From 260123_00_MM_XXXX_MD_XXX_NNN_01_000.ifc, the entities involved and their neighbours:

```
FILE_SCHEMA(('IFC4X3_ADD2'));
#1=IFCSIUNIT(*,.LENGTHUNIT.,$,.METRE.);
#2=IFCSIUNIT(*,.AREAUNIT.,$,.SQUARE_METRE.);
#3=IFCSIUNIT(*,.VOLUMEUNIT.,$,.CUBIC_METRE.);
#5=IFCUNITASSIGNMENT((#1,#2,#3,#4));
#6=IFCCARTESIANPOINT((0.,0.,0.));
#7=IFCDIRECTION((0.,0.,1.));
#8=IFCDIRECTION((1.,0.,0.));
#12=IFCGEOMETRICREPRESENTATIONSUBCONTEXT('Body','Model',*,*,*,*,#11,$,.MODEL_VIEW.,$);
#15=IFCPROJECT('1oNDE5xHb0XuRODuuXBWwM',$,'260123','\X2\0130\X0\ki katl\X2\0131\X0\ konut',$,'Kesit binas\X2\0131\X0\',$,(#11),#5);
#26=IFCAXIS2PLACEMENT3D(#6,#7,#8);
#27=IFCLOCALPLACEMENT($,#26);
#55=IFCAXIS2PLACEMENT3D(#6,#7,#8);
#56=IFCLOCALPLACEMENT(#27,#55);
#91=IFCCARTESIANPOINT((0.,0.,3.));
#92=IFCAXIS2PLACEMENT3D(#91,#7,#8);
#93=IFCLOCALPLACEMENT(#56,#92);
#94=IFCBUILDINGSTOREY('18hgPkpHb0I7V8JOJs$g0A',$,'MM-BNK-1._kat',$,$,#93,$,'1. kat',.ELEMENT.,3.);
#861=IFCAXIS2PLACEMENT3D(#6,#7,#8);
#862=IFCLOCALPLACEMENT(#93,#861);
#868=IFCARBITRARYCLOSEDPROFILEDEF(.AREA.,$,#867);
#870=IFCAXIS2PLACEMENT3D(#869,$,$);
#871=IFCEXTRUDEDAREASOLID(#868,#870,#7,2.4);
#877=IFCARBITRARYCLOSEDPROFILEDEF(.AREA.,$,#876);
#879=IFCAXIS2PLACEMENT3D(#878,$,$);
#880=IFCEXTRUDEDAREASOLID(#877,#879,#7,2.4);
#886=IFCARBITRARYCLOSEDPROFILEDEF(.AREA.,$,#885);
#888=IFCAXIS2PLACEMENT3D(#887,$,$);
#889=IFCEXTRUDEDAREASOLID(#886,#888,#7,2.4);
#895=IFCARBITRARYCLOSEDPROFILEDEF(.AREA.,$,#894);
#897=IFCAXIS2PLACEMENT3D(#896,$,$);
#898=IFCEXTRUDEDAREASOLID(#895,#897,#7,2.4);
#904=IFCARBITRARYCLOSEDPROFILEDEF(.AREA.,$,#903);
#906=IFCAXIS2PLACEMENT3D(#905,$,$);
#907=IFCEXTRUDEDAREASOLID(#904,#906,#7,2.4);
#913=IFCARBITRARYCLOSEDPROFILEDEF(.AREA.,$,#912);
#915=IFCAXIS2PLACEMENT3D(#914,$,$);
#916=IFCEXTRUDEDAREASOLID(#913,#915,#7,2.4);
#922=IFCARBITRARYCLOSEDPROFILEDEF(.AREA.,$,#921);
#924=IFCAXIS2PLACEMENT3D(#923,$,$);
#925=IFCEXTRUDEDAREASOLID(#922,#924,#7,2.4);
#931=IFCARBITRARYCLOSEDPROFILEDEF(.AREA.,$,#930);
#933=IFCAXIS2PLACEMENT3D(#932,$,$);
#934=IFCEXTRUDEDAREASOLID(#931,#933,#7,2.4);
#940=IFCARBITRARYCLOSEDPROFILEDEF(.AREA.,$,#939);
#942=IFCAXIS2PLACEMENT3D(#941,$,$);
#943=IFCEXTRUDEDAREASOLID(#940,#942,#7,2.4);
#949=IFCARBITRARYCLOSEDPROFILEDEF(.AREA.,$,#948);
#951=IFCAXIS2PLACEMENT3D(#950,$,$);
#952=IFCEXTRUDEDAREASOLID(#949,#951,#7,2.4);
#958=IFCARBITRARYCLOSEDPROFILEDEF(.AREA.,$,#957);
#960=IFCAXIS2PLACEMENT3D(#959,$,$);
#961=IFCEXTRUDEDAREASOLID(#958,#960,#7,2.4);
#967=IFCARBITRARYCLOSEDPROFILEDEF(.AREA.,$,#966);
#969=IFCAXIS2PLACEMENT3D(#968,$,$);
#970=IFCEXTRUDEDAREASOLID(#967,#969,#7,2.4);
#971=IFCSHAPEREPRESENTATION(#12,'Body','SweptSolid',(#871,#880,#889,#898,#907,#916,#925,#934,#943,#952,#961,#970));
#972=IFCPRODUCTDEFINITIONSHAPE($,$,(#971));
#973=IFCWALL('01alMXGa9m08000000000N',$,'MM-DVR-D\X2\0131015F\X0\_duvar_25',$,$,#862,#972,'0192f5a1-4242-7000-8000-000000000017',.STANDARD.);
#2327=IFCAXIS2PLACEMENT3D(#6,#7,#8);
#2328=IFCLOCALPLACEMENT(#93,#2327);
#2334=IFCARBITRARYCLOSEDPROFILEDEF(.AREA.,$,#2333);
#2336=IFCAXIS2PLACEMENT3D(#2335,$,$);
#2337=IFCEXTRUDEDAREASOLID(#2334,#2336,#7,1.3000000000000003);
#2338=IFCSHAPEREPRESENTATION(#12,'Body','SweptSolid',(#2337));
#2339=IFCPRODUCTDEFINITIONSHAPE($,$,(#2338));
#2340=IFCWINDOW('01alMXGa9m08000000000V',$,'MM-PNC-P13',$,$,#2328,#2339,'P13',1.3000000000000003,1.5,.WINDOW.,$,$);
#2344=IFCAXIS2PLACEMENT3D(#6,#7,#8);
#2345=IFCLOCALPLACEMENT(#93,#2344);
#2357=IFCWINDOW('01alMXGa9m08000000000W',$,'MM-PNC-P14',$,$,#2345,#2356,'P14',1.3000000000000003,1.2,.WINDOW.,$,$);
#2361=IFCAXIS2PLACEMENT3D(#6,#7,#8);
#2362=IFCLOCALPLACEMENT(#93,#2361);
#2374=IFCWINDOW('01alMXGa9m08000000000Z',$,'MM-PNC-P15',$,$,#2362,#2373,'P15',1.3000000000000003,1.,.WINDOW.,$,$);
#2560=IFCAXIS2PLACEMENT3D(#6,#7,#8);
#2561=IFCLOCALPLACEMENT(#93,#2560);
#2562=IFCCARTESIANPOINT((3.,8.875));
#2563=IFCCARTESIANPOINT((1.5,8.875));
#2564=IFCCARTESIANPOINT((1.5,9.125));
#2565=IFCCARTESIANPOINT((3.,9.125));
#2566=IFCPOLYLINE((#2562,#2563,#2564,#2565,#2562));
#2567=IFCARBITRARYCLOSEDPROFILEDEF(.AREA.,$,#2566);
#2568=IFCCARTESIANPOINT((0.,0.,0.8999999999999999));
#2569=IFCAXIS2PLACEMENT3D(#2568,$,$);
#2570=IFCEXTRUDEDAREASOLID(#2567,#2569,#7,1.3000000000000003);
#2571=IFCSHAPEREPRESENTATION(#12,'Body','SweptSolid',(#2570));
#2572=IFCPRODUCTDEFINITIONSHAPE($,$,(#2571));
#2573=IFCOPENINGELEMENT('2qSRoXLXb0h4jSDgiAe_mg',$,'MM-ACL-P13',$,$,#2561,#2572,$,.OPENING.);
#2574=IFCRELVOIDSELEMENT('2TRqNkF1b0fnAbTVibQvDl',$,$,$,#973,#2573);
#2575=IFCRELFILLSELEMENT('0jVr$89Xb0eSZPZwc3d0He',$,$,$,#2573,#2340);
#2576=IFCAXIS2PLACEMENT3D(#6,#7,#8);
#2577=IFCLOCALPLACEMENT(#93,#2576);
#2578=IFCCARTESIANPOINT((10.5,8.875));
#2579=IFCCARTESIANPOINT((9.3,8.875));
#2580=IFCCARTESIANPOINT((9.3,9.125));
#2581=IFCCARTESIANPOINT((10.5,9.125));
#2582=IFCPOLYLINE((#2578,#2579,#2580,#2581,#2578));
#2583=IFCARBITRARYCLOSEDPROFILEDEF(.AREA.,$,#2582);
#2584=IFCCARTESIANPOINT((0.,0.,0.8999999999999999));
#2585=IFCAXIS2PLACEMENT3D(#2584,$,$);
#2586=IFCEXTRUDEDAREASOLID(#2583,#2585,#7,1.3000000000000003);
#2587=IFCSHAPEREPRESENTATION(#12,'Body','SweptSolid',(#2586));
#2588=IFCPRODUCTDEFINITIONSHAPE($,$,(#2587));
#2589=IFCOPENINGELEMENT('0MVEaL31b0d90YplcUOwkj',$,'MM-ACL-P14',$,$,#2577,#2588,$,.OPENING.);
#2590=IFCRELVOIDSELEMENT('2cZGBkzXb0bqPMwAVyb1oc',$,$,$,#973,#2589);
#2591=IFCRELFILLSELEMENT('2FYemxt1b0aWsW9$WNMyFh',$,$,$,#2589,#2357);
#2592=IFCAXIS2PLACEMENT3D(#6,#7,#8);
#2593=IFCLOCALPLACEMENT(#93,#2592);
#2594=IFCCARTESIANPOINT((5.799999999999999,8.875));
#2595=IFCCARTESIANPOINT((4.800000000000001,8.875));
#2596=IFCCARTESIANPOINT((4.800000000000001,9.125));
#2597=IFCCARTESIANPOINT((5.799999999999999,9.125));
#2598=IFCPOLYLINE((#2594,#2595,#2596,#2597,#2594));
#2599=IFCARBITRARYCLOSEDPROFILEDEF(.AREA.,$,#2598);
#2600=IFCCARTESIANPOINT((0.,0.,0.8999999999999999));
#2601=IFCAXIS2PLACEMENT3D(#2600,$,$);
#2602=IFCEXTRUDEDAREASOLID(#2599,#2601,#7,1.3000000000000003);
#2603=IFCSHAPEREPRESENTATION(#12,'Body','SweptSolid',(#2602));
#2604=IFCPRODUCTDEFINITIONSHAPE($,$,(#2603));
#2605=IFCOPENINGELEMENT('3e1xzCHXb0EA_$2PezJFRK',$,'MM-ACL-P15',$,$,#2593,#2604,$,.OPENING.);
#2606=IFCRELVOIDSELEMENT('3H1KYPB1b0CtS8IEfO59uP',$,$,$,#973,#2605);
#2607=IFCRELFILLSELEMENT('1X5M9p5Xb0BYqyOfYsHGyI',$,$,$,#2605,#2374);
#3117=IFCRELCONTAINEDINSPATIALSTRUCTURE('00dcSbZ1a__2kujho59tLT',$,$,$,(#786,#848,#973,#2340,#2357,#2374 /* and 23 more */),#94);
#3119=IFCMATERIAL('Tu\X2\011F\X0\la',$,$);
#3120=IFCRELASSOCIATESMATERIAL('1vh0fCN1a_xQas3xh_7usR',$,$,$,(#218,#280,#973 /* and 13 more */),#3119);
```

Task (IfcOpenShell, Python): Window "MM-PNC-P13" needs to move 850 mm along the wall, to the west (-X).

```python
import ifcopenshell
import ifcopenshell.api.geometry
import ifcopenshell.util.placement
import ifcopenshell.util.unit

model = ifcopenshell.open("260123_00_MM_XXXX_MD_XXX_NNN_01_000.ifc")
unit_scale = ifcopenshell.util.unit.calculate_unit_scale(model)

window = model.by_guid("01alMXGa9m08000000000V")
opening = window.FillsVoids[0].RelatingOpeningElement
wall = opening.VoidsElements[0].RelatingBuildingElement

wall_matrix = ifcopenshell.util.placement.get_local_placement(wall.ObjectPlacement)
shift = wall_matrix[:3, 0] * -0.85 / unit_scale
before = ifcopenshell.util.placement.get_local_placement(window.ObjectPlacement)[:3, 3].copy()

# The window is not placed relative to its opening, so move both.
for product in (opening, window):
    matrix = ifcopenshell.util.placement.get_local_placement(product.ObjectPlacement)
    matrix[:3, 3] += shift
    ifcopenshell.api.geometry.edit_object_placement(model, product=product, matrix=matrix, is_si=False)

after = ifcopenshell.util.placement.get_local_placement(window.ObjectPlacement)[:3, 3]
print("window moved by", (after - before).round(3) + 0.0)

model.write("260123_00_MM_XXXX_MD_XXX_NNN_01_000-out.ifc")
```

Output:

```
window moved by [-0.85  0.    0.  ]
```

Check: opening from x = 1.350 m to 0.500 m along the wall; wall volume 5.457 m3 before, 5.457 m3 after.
